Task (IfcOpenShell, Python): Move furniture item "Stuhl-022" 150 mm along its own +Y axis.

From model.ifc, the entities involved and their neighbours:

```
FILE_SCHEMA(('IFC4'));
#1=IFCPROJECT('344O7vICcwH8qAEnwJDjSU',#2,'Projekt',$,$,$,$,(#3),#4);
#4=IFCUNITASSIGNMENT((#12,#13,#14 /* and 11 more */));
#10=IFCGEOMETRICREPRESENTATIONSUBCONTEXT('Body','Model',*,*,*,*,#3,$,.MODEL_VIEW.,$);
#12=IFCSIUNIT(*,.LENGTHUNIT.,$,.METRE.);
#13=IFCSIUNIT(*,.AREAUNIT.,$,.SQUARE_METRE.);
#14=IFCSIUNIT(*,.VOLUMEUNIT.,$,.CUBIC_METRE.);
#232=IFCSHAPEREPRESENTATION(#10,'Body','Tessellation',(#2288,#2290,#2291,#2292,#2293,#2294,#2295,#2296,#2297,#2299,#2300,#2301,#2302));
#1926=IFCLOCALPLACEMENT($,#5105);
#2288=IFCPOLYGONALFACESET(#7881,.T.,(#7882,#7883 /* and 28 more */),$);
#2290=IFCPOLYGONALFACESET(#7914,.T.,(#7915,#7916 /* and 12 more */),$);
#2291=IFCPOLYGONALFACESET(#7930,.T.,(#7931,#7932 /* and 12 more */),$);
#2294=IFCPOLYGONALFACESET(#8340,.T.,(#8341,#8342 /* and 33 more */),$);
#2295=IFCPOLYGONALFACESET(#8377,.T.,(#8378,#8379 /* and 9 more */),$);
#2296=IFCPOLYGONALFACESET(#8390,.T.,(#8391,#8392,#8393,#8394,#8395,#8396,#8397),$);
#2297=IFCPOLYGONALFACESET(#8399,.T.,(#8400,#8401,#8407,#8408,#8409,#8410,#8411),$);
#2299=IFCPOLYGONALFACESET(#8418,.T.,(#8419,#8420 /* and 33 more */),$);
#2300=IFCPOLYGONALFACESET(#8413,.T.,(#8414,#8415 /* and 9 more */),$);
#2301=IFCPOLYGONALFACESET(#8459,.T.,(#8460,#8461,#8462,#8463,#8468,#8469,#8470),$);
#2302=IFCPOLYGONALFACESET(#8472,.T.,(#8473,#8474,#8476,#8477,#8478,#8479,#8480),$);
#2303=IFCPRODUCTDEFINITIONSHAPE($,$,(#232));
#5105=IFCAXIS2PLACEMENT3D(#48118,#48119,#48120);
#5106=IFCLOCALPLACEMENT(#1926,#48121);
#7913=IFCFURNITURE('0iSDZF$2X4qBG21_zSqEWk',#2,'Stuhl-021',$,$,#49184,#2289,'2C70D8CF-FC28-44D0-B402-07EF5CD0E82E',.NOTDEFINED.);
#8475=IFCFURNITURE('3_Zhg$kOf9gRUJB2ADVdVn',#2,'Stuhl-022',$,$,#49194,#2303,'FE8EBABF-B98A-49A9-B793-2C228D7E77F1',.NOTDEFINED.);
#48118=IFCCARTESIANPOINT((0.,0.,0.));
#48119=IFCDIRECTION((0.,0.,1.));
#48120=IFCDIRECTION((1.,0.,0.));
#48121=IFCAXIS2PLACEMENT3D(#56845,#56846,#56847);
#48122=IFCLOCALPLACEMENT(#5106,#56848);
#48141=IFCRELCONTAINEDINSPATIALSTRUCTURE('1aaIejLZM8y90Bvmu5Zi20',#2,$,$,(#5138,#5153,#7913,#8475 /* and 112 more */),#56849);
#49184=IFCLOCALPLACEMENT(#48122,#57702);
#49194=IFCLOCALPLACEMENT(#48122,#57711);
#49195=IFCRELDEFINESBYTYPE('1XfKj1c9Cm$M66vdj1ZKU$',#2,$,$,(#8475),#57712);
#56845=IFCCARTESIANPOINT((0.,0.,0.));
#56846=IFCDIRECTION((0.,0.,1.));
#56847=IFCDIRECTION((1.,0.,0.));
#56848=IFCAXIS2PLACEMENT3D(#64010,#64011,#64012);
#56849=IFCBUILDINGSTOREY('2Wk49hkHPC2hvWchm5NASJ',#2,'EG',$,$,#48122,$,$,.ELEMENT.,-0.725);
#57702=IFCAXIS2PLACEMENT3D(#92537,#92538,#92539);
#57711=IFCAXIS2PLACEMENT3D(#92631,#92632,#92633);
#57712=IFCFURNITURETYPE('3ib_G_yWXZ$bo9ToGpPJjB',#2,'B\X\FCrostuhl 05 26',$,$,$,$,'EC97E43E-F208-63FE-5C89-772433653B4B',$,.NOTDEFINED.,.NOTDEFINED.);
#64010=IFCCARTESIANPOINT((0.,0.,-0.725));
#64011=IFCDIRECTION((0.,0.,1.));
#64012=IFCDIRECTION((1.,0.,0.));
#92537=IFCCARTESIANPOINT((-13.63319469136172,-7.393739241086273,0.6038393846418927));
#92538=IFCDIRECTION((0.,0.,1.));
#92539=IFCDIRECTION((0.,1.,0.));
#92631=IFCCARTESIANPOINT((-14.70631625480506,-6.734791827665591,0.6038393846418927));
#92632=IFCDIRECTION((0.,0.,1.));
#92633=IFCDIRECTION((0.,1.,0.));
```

```python
import ifcopenshell
import ifcopenshell.api.geometry
import ifcopenshell.util.placement
import ifcopenshell.util.unit

model = ifcopenshell.open("model.ifc")
unit_scale = ifcopenshell.util.unit.calculate_unit_scale(model)

item = model.by_guid("3_Zhg$kOf9gRUJB2ADVdVn")
matrix = ifcopenshell.util.placement.get_local_placement(item.ObjectPlacement)
matrix[:3, 3] += matrix[:3, 1] * 0.15 / unit_scale
ifcopenshell.api.geometry.edit_object_placement(model, product=item, matrix=matrix, is_si=False)

print(ifcopenshell.util.placement.get_local_placement(item.ObjectPlacement).round(3) + 0.0)

model.write("model-out.ifc")
```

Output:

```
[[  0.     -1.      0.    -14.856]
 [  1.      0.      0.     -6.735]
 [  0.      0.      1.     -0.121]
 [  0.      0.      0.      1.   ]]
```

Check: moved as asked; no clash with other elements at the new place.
